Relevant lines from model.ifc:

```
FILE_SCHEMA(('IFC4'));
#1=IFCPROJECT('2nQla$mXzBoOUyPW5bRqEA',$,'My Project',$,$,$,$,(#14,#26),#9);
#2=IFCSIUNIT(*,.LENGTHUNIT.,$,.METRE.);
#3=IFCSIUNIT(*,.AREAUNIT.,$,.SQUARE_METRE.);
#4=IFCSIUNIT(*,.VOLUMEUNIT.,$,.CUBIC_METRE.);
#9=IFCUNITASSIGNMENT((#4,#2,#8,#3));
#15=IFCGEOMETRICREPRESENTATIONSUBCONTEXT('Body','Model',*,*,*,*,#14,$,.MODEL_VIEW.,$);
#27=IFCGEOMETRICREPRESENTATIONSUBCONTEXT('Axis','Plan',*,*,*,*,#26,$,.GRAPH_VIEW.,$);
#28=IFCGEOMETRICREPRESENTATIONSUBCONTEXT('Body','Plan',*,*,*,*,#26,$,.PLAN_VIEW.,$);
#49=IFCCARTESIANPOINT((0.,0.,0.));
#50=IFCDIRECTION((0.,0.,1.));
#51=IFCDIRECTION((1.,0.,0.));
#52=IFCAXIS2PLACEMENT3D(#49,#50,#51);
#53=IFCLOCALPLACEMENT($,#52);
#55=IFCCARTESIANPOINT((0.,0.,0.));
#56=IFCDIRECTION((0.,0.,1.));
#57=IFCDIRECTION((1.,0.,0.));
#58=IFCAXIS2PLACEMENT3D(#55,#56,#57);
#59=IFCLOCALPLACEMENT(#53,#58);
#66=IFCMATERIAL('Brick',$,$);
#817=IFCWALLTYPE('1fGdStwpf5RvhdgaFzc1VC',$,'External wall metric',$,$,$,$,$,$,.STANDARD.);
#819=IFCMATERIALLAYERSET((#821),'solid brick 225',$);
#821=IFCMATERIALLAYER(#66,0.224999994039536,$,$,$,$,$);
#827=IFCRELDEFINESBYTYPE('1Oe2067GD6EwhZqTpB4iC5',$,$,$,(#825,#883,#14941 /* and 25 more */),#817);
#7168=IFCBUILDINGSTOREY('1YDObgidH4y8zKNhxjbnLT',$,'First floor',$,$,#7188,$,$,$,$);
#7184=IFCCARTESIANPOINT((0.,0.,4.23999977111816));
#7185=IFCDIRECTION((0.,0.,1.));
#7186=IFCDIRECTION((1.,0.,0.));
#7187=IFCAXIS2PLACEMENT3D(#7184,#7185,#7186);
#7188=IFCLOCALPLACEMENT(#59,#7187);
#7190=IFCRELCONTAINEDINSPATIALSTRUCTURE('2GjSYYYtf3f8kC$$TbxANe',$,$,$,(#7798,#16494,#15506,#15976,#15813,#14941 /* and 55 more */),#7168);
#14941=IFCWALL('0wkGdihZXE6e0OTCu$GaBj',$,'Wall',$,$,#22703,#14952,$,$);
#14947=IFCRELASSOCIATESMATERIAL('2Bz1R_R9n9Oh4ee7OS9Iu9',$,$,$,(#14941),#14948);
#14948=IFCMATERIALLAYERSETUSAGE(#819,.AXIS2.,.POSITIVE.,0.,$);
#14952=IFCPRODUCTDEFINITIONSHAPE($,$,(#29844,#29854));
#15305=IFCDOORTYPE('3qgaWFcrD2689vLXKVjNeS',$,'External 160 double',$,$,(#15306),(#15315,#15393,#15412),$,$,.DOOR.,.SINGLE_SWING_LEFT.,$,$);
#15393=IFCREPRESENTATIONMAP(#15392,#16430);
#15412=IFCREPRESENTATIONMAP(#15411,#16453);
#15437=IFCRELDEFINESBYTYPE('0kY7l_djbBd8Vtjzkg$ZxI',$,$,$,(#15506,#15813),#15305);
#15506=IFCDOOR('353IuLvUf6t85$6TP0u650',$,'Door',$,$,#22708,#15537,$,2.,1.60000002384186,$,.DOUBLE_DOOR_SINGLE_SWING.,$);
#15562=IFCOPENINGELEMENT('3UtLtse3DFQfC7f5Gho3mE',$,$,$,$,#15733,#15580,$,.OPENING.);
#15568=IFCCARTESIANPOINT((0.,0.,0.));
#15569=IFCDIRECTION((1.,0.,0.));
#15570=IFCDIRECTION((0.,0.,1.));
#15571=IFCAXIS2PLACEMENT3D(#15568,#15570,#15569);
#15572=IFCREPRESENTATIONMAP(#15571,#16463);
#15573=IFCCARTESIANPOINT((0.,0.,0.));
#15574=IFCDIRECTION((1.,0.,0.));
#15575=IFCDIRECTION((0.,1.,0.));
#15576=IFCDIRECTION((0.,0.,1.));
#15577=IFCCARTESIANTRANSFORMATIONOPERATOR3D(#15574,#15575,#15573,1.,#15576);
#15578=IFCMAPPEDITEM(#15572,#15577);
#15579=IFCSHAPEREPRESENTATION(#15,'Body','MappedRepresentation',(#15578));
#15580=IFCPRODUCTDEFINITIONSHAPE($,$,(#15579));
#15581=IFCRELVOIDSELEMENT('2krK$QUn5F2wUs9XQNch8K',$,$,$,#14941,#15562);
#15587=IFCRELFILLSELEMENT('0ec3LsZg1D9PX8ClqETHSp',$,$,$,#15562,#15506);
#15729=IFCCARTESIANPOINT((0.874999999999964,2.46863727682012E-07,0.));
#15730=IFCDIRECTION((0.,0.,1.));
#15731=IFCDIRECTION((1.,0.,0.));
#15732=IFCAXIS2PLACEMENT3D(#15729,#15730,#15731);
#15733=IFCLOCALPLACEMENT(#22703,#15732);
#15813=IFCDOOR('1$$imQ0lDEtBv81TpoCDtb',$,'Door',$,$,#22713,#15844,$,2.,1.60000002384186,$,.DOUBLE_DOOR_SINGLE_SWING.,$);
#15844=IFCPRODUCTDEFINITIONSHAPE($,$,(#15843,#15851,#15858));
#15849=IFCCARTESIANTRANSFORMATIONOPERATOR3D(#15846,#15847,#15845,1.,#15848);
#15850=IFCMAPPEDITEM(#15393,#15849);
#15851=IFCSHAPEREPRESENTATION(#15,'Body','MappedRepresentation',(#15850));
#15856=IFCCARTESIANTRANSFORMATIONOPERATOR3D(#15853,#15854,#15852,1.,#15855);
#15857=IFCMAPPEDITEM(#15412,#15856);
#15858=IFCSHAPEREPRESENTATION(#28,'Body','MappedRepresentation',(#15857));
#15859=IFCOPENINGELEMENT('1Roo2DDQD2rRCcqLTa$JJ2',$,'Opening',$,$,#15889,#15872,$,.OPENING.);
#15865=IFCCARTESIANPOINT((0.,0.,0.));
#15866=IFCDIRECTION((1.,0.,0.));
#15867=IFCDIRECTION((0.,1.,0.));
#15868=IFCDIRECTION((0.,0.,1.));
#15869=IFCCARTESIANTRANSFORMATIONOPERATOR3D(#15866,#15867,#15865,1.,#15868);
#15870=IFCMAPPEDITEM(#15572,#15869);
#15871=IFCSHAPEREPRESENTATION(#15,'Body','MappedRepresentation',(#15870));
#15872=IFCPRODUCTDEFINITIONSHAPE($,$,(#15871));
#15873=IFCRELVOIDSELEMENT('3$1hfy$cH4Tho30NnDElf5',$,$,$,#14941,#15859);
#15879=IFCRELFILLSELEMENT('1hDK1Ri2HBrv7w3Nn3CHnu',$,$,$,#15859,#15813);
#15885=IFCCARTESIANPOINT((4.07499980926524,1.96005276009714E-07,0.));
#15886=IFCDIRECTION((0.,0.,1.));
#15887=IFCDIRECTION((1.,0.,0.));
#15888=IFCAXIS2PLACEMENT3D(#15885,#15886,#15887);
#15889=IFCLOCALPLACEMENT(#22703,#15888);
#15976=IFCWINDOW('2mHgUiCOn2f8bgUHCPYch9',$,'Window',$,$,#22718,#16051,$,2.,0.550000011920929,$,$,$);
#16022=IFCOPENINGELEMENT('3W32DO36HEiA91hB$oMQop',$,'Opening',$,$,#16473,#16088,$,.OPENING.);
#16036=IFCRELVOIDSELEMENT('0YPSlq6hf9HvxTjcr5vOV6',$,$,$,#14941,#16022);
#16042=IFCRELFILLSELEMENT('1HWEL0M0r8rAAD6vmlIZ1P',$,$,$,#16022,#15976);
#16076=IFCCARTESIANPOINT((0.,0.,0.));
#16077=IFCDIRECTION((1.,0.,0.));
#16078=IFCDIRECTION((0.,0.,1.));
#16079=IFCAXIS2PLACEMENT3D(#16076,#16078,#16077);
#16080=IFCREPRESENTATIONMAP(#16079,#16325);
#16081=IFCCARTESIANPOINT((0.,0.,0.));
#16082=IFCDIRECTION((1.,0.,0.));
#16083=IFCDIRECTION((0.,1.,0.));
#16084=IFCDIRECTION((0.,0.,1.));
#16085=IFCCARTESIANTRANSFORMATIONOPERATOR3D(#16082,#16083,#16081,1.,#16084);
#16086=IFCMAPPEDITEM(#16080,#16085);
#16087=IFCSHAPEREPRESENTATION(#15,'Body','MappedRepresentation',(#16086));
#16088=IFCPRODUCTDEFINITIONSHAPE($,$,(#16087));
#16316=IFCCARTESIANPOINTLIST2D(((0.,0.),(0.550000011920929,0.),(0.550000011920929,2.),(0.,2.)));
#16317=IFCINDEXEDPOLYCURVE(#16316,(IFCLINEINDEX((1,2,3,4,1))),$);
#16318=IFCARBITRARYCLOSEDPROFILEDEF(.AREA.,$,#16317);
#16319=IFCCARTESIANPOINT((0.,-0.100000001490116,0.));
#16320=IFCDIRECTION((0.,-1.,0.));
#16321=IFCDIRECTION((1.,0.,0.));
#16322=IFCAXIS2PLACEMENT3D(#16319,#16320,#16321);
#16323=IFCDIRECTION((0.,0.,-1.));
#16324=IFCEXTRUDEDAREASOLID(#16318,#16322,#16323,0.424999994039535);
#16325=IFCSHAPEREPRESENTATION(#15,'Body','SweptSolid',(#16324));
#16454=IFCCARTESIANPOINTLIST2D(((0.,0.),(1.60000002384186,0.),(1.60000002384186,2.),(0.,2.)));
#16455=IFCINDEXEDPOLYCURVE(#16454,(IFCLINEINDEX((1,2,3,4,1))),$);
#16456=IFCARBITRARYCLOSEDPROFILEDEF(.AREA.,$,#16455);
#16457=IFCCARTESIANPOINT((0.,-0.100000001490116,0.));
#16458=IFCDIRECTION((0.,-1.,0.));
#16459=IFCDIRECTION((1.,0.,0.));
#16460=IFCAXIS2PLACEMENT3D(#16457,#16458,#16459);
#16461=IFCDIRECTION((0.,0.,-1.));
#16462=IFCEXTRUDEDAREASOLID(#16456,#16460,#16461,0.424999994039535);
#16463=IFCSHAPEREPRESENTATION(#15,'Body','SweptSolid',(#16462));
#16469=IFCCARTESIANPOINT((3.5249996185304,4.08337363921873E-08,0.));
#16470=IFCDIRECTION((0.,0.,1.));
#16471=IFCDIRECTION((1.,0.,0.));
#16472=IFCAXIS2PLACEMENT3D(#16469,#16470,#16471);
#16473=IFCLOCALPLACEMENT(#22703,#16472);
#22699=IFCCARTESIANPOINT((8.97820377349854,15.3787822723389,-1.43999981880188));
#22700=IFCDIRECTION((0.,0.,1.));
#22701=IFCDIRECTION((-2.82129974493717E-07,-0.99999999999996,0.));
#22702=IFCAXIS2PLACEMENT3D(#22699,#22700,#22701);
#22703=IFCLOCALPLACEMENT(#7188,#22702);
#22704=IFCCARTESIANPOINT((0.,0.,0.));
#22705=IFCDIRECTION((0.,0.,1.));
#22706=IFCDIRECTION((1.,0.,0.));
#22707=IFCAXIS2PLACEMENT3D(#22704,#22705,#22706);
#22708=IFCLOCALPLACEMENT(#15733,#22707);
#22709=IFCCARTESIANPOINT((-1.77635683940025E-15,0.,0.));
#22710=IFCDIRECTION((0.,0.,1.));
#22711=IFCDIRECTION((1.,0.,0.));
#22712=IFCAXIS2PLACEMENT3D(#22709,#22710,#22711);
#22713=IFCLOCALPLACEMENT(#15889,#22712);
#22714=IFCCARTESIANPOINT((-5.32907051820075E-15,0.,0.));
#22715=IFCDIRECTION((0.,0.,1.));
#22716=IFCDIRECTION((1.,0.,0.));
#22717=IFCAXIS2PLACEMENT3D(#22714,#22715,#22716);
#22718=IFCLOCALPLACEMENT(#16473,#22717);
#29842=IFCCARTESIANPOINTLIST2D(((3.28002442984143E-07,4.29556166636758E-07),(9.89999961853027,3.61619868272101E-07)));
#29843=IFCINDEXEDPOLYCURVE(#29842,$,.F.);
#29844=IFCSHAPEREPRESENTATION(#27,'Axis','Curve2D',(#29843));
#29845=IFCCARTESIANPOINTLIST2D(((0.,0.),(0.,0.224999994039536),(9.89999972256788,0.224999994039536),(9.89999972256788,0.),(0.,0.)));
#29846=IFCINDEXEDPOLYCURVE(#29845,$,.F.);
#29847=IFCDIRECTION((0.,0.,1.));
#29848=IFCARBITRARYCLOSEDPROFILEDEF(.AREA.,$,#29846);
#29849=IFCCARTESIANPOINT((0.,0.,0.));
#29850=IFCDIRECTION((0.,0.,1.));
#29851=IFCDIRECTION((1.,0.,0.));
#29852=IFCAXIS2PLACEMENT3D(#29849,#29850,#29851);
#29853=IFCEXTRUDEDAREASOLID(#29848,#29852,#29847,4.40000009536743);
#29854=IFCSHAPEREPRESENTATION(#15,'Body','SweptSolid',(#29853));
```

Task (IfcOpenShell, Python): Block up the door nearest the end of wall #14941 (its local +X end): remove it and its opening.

```python
import ifcopenshell
import ifcopenshell.api.feature
import ifcopenshell.api.root
import ifcopenshell.geom
import ifcopenshell.util.shape

model = ifcopenshell.open("model.ifc")
settings = ifcopenshell.geom.settings()


def volume(element):
    """Net volume in cubic metres, openings subtracted."""
    shape = ifcopenshell.geom.create_shape(settings, element)
    return ifcopenshell.util.shape.get_volume(shape.geometry)


door = model.by_guid("1$$imQ0lDEtBv81TpoCDtb")
opening = door.FillsVoids[0].RelatingOpeningElement
wall = opening.VoidsElements[0].RelatingBuildingElement
before = volume(wall)

ifcopenshell.api.root.remove_product(model, product=door)
ifcopenshell.api.feature.remove_feature(model, feature=opening)

after = volume(wall)

print(f"wall volume {before:.3f} -> {after:.3f} m3")

model.write("model_v2.ifc")
```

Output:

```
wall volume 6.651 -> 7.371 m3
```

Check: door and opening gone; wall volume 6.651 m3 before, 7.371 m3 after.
